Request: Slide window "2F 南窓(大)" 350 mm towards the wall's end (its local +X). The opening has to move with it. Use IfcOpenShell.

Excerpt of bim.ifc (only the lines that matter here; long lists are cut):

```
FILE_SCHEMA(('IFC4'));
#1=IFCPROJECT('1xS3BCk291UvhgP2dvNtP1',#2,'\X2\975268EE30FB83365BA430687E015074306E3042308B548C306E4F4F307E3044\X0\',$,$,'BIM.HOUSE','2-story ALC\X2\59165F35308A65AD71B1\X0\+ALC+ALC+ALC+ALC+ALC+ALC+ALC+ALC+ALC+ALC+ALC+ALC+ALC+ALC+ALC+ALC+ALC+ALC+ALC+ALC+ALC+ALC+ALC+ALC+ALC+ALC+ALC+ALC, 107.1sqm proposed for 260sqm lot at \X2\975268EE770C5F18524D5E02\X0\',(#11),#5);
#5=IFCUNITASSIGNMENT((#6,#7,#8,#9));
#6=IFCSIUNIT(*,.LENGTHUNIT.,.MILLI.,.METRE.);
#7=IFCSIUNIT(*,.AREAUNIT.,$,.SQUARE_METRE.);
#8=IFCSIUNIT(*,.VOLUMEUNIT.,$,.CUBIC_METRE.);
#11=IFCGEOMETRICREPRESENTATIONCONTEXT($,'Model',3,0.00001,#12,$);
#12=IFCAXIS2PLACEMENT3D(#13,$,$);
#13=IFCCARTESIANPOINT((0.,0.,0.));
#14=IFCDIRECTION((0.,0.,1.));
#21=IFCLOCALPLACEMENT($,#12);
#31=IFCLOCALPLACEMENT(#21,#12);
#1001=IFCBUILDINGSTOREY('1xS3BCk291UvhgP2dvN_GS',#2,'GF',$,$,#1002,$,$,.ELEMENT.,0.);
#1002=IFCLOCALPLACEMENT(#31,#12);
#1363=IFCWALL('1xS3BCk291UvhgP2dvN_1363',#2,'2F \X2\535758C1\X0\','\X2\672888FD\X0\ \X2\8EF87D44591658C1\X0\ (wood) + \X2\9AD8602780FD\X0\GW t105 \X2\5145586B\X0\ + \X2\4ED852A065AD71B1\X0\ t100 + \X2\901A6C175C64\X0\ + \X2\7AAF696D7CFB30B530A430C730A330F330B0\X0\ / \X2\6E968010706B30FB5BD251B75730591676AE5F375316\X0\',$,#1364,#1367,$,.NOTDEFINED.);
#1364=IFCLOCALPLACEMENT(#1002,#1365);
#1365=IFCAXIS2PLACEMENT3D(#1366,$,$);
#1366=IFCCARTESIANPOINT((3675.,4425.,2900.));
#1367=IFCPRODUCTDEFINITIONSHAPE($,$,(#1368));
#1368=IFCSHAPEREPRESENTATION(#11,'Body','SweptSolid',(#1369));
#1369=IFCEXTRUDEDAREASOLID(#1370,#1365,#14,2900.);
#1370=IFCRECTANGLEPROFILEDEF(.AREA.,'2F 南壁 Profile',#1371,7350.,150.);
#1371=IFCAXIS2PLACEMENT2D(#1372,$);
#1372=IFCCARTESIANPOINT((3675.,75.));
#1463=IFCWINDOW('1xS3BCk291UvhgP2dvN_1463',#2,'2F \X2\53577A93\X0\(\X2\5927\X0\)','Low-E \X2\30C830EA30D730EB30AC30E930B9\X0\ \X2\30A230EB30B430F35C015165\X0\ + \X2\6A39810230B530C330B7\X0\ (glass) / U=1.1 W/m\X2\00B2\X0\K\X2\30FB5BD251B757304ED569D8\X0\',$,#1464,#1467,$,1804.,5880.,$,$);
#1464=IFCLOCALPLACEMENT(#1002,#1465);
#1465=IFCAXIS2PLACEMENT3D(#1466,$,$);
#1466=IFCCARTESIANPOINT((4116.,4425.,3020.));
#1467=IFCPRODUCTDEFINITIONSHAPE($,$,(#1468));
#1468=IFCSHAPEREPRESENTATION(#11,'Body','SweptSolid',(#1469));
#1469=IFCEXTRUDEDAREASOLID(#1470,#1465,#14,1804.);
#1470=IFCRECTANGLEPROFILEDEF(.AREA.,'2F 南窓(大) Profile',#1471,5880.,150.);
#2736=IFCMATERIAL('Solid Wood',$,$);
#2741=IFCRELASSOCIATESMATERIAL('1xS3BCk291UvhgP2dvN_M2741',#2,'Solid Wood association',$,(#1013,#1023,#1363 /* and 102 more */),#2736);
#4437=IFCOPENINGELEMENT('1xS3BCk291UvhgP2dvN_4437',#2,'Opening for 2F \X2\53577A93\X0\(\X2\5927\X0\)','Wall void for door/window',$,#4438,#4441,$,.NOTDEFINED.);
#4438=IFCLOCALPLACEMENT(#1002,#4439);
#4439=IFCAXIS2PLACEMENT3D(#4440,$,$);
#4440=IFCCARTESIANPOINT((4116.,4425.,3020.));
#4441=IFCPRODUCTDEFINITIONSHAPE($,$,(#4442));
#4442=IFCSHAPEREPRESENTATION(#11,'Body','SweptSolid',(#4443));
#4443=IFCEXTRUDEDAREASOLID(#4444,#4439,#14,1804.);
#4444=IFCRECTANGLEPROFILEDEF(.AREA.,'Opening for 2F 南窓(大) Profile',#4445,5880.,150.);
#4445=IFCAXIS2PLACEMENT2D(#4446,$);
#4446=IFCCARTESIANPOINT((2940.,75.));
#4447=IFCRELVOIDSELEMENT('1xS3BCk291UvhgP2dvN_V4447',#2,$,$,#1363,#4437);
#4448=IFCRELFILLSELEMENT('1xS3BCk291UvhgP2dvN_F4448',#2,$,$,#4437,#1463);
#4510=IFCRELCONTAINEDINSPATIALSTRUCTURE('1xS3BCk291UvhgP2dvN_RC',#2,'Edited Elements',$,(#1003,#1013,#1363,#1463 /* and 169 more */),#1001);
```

```python
import ifcopenshell
import ifcopenshell.api.geometry
import ifcopenshell.util.placement

model = ifcopenshell.open("bim.ifc")

window = model.by_guid("1xS3BCk291UvhgP2dvN_1463")
opening = window.FillsVoids[0].RelatingOpeningElement
wall = opening.VoidsElements[0].RelatingBuildingElement

wall_matrix = ifcopenshell.util.placement.get_local_placement(wall.ObjectPlacement)
shift = wall_matrix[:3, 0] * 350.0
before = ifcopenshell.util.placement.get_local_placement(window.ObjectPlacement)[:3, 3].copy()

# The window is not placed relative to its opening, so move both.
for product in (opening, window):
    matrix = ifcopenshell.util.placement.get_local_placement(product.ObjectPlacement)
    matrix[:3, 3] += shift
    ifcopenshell.api.geometry.edit_object_placement(model, product=product, matrix=matrix, is_si=False)

after = ifcopenshell.util.placement.get_local_placement(window.ObjectPlacement)[:3, 3]
print("window moved by", (after - before).round(3) + 0.0)

model.write("bim_rev.ifc")
```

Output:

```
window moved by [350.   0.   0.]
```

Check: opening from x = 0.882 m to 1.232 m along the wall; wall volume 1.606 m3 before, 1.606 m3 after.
